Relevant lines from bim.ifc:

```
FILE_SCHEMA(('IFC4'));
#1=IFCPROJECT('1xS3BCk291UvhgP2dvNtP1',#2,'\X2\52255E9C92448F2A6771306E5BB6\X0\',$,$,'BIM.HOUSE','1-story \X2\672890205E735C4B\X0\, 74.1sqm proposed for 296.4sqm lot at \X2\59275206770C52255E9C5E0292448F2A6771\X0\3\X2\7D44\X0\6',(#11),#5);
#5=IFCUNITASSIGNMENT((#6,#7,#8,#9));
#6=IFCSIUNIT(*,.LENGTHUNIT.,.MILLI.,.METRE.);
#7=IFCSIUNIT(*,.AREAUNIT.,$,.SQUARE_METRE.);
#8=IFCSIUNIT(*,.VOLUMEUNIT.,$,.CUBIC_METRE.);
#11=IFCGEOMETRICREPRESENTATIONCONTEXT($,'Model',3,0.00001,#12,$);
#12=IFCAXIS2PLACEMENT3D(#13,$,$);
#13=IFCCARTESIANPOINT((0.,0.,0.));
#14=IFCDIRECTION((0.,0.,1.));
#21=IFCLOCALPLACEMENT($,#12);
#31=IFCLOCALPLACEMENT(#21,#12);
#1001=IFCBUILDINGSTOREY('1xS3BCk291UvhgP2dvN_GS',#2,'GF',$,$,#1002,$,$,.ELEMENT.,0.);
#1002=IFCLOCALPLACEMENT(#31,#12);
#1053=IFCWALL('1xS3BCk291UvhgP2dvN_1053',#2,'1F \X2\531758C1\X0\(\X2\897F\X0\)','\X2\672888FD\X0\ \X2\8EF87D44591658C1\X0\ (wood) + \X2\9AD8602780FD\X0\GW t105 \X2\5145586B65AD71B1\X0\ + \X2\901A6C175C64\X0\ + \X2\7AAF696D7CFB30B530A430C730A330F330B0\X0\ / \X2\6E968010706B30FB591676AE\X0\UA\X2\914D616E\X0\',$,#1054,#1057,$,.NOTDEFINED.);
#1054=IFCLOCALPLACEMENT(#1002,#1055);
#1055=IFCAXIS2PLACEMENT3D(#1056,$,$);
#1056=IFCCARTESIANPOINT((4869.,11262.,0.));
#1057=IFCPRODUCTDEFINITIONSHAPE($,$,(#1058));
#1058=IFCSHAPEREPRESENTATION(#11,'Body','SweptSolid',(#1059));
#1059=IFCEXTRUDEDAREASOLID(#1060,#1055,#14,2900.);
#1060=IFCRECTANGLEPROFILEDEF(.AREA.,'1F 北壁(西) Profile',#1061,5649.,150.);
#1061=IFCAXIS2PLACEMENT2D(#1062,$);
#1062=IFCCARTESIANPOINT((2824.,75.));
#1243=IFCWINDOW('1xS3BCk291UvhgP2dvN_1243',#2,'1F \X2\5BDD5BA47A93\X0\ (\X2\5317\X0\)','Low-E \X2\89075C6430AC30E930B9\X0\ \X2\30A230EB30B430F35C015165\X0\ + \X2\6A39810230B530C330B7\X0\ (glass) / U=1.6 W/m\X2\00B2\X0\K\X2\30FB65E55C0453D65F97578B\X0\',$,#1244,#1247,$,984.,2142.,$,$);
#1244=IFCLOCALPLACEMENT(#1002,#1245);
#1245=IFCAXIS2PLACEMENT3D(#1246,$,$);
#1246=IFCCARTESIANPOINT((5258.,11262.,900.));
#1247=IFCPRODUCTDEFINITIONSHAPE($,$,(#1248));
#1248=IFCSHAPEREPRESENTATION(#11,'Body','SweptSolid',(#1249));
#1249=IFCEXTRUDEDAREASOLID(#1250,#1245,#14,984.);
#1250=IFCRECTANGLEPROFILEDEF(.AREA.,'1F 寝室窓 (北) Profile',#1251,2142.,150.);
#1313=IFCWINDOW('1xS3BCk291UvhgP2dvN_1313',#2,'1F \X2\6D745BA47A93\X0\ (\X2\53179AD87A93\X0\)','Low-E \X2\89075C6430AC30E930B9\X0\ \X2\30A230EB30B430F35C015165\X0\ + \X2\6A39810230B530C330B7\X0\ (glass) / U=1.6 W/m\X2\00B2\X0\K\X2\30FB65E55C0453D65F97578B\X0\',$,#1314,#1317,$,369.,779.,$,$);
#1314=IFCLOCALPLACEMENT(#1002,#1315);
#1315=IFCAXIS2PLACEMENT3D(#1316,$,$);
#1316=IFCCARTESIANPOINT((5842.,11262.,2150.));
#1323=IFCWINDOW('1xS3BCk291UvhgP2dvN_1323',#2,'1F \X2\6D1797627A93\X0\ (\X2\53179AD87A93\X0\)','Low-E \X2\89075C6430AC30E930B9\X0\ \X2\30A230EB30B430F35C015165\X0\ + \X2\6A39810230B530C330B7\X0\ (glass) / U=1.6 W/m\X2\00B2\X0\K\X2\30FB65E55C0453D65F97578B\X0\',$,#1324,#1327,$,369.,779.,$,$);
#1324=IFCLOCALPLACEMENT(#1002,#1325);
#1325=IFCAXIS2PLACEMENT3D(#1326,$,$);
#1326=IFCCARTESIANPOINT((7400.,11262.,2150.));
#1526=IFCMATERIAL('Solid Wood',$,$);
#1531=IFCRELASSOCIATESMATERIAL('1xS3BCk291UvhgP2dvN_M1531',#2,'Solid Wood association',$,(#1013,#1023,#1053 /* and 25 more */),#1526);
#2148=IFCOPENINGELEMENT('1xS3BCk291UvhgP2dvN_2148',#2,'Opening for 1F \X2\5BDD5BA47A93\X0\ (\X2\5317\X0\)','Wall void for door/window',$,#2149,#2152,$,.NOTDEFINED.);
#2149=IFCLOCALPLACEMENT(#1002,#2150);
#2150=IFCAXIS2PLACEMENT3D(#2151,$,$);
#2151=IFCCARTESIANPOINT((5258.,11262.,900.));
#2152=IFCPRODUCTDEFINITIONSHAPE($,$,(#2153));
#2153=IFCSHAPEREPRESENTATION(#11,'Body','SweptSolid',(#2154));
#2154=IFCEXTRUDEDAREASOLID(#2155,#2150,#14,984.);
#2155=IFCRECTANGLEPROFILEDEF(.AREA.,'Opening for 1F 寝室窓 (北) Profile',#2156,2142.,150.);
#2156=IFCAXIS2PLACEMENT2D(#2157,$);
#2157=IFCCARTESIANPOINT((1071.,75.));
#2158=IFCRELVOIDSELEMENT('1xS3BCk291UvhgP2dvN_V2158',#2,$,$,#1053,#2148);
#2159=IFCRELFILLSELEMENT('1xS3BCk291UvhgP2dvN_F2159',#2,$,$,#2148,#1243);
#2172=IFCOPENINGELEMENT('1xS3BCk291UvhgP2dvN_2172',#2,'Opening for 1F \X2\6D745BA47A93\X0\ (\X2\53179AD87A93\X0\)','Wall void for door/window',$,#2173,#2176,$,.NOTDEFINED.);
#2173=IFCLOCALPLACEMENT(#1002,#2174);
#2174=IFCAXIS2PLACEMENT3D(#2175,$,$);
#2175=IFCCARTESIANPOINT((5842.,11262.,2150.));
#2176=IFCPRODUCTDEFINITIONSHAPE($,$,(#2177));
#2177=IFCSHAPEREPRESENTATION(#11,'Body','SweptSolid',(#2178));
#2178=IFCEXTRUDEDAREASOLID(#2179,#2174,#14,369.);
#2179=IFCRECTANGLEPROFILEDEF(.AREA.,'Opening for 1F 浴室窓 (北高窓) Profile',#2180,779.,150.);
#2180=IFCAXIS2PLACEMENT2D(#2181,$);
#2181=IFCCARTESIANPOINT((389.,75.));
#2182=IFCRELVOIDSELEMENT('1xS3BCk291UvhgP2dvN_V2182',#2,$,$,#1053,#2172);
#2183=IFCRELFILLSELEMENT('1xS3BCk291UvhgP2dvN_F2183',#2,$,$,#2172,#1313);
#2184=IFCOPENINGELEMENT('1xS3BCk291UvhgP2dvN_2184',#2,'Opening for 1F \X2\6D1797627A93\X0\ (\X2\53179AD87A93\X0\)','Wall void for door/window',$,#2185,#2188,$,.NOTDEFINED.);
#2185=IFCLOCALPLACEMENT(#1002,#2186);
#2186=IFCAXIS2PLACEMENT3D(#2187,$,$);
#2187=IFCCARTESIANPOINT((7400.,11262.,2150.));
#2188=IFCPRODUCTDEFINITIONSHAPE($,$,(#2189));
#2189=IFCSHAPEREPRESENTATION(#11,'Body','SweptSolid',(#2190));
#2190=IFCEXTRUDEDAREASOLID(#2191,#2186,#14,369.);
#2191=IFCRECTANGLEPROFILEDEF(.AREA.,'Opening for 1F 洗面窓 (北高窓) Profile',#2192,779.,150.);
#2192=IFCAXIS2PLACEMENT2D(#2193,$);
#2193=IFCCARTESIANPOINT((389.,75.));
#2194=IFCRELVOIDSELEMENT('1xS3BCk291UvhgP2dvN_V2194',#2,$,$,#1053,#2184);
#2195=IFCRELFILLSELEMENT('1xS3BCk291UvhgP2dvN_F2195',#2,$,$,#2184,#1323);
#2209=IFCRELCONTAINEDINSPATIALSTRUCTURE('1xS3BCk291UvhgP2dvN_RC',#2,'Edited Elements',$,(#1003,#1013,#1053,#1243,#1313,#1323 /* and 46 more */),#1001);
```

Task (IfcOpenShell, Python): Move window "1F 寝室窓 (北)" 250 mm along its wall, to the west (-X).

```python
import ifcopenshell
import ifcopenshell.api.geometry
import ifcopenshell.util.placement
import ifcopenshell.util.unit

model = ifcopenshell.open("bim.ifc")
unit_scale = ifcopenshell.util.unit.calculate_unit_scale(model)

window = model.by_id(1243)
opening = window.FillsVoids[0].RelatingOpeningElement
wall = opening.VoidsElements[0].RelatingBuildingElement

wall_matrix = ifcopenshell.util.placement.get_local_placement(wall.ObjectPlacement)
shift = wall_matrix[:3, 0] * -0.25 / unit_scale
before = ifcopenshell.util.placement.get_local_placement(window.ObjectPlacement)[:3, 3].copy()

# The window is not placed relative to its opening, so move both.
for product in (opening, window):
    matrix = ifcopenshell.util.placement.get_local_placement(product.ObjectPlacement)
    matrix[:3, 3] += shift
    ifcopenshell.api.geometry.edit_object_placement(model, product=product, matrix=matrix, is_si=False)

after = ifcopenshell.util.placement.get_local_placement(window.ObjectPlacement)[:3, 3]
print("window moved by", (after - before).round(3) + 0.0)

model.write("bim_v2.ifc")
```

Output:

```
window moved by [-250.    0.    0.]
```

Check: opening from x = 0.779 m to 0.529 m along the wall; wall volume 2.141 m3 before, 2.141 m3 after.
